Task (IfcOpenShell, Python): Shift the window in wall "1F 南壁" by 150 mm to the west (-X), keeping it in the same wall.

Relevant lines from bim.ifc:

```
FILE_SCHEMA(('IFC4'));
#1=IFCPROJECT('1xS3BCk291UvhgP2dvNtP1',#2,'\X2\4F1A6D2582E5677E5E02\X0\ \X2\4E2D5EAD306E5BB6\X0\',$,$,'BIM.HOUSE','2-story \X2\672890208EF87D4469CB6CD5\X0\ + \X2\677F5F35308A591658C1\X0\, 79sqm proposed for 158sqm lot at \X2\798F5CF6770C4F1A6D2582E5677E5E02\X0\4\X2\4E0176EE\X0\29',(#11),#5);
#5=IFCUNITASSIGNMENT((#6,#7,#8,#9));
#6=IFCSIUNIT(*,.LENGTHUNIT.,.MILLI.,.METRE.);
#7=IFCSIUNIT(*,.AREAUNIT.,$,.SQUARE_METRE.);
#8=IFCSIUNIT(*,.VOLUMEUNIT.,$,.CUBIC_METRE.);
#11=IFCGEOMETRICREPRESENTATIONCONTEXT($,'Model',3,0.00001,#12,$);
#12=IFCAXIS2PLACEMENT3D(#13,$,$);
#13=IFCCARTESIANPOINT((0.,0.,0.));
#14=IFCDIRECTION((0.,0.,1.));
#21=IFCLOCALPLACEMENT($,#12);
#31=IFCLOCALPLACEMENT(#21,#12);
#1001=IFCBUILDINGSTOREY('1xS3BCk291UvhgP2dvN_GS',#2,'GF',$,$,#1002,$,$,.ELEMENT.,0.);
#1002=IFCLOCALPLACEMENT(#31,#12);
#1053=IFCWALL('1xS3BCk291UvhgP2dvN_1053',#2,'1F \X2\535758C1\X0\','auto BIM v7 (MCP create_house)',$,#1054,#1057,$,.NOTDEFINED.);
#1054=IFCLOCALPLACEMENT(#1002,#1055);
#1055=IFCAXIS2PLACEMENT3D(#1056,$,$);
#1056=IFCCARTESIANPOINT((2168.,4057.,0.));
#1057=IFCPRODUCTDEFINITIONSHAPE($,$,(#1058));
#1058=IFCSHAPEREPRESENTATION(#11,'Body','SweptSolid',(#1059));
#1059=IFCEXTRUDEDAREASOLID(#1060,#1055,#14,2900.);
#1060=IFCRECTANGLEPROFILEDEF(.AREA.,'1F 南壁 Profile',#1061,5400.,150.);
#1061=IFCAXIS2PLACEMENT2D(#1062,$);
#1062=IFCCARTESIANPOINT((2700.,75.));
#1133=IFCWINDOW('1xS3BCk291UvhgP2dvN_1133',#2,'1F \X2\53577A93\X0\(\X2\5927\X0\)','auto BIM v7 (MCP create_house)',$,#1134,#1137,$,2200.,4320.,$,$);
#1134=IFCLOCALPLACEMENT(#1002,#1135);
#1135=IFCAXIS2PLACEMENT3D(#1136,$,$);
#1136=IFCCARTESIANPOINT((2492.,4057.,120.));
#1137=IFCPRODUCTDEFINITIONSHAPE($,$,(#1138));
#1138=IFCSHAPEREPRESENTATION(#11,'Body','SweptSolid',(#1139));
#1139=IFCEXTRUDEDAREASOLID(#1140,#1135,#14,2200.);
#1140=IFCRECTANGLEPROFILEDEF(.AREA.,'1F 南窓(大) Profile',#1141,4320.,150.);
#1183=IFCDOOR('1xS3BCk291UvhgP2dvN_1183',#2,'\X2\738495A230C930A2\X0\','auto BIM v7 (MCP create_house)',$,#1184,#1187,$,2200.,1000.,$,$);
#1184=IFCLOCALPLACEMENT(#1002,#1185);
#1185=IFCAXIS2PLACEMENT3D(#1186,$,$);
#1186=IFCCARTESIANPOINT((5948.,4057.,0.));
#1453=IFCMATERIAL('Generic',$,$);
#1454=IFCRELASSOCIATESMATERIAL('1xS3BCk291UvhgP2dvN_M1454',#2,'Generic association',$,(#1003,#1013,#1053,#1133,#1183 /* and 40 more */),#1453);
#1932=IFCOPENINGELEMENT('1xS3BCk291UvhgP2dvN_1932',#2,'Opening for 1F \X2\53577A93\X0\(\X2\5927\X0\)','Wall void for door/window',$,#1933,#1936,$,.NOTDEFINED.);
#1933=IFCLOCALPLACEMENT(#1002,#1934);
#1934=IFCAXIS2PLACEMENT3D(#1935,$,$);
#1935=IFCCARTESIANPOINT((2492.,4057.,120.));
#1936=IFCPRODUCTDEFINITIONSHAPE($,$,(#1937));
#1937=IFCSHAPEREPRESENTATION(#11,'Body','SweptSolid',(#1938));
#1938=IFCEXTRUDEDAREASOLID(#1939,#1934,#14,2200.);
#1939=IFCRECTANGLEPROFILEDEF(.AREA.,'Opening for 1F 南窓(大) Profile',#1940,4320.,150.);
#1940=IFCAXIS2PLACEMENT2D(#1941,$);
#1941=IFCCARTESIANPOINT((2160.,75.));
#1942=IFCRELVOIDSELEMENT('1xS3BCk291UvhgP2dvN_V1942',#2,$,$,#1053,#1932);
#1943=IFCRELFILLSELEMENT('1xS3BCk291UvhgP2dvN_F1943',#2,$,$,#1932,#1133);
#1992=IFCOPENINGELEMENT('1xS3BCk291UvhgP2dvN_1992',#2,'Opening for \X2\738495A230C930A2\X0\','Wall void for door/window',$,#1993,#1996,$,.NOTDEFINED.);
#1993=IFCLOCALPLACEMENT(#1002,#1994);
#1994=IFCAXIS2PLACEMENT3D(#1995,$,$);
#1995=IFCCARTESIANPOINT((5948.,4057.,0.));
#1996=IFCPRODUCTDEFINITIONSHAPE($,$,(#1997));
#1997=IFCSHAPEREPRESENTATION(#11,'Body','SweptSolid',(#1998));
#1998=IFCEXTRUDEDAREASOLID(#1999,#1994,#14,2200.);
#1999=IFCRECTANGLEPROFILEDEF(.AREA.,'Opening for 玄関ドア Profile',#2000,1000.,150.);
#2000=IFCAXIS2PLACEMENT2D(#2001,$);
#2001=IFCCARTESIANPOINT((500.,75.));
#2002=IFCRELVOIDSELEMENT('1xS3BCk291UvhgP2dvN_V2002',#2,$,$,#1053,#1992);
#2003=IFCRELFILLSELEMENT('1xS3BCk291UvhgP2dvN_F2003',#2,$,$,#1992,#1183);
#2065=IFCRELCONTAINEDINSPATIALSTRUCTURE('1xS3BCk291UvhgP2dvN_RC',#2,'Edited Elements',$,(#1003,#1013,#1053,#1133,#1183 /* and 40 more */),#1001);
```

```python
import ifcopenshell
import ifcopenshell.api.geometry
import ifcopenshell.util.placement
import ifcopenshell.util.unit

model = ifcopenshell.open("bim.ifc")
unit_scale = ifcopenshell.util.unit.calculate_unit_scale(model)

window = model.by_guid("1xS3BCk291UvhgP2dvN_1133")
opening = window.FillsVoids[0].RelatingOpeningElement
wall = opening.VoidsElements[0].RelatingBuildingElement

wall_matrix = ifcopenshell.util.placement.get_local_placement(wall.ObjectPlacement)
shift = wall_matrix[:3, 0] * -0.15 / unit_scale
before = ifcopenshell.util.placement.get_local_placement(window.ObjectPlacement)[:3, 3].copy()

# The window is not placed relative to its opening, so move both.
for product in (opening, window):
    matrix = ifcopenshell.util.placement.get_local_placement(product.ObjectPlacement)
    matrix[:3, 3] += shift
    ifcopenshell.api.geometry.edit_object_placement(model, product=product, matrix=matrix, is_si=False)

after = ifcopenshell.util.placement.get_local_placement(window.ObjectPlacement)[:3, 3]
print("window moved by", (after - before).round(3) + 0.0)

model.write("bim-out.ifc")
```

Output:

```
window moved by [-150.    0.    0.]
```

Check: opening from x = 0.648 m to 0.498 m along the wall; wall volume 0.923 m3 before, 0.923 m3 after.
